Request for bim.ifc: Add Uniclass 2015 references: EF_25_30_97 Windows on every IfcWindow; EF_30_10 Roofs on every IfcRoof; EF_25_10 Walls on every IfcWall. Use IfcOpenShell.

First a look at what the model holds.

```python
import ifcopenshell

model = ifcopenshell.open("bim.ifc")
print(model.schema)
print("classifications:", [c.Name for c in model.by_type("IfcClassification")])
for ifc_class in ("IfcDoor", "IfcRoof", "IfcStair", "IfcWall", "IfcWindow"):
    print(ifc_class, len(model.by_type(ifc_class)))
```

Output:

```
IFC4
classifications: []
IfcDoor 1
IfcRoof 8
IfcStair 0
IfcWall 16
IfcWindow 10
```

```python
import ifcopenshell
import ifcopenshell.api.classification

model = ifcopenshell.open("bim.ifc")

system = ifcopenshell.api.classification.add_classification(model, classification="Uniclass 2015")

codes = {
    "IfcWindow": ("EF_25_30_97", "Windows"),
    "IfcRoof": ("EF_30_10", "Roofs"),
    "IfcWall": ("EF_25_10", "Walls"),
}
for ifc_class, (code, name) in codes.items():
    products = model.by_type(ifc_class)
    ifcopenshell.api.classification.add_reference(
        model, products=products, classification=system, identification=code, name=name
    )
    print(code, len(products))

model.write("bim-out.ifc")
```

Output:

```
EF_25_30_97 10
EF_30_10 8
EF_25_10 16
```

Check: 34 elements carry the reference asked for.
